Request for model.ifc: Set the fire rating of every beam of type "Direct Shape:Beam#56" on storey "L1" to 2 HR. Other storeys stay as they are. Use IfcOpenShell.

First a look at what the model holds.

```python
import ifcopenshell
import ifcopenshell.util.element

model = ifcopenshell.open("model.ifc")
print(model.schema)
storey = next(s for s in model.by_type("IfcBuildingStorey") if s.Name == "L1")
beams = [e for e in ifcopenshell.util.element.get_decomposition(storey) if e.is_a("IfcBeam")]
seen = {}
for e in beams:
    element_type = ifcopenshell.util.element.get_type(e)
    key = (element_type.Name if element_type != e and element_type else None, ifcopenshell.util.element.get_pset(e, "Pset_BeamCommon", "FireRating"))
    seen[key] = seen.get(key, 0) + 1
for (name, value), count in sorted(seen.items(), key=str):
    print(count, "x", name, "|", value)
```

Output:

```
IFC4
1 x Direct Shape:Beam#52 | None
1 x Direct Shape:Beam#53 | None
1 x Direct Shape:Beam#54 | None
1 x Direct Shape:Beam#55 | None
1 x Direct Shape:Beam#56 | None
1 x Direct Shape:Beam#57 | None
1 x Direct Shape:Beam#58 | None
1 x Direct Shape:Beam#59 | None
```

```python
import ifcopenshell
import ifcopenshell.api.pset
import ifcopenshell.util.element

model = ifcopenshell.open("model.ifc")

storey = next(s for s in model.by_type("IfcBuildingStorey") if s.Name == "L1")
beams = [e for e in ifcopenshell.util.element.get_decomposition(storey) if e.is_a("IfcBeam")]

count = 0
for e in beams:
    element_type = ifcopenshell.util.element.get_type(e)
    if element_type in (None, e) or element_type.Name != "Direct Shape:Beam#56":
        continue
    # add_pset returns the element's existing set when there is one.
    pset = ifcopenshell.api.pset.add_pset(model, product=e, name="Pset_BeamCommon")
    ifcopenshell.api.pset.edit_pset(model, pset=pset, properties={"FireRating": "2 HR"})
    count += 1

print(count, "beams updated")

model.write("model_v2.ifc")
```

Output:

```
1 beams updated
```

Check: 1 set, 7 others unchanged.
